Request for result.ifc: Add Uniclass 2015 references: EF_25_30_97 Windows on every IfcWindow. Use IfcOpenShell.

First a look at what the model holds.

```python
import ifcopenshell

model = ifcopenshell.open("result.ifc")
print(model.schema)
print("classifications:", [c.Name for c in model.by_type("IfcClassification")])
for ifc_class in ("IfcDoor", "IfcRoof", "IfcStair", "IfcWall", "IfcWindow"):
    print(ifc_class, len(model.by_type(ifc_class)))
```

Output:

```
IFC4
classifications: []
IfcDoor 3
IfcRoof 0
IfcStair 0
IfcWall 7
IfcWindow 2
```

```python
import ifcopenshell
import ifcopenshell.api.classification

model = ifcopenshell.open("result.ifc")

system = ifcopenshell.api.classification.add_classification(model, classification="Uniclass 2015")

codes = {
    "IfcWindow": ("EF_25_30_97", "Windows"),
}
for ifc_class, (code, name) in codes.items():
    products = model.by_type(ifc_class)
    ifcopenshell.api.classification.add_reference(
        model, products=products, classification=system, identification=code, name=name
    )
    print(code, len(products))

model.write("result_v2.ifc")
```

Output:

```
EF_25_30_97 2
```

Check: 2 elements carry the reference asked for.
